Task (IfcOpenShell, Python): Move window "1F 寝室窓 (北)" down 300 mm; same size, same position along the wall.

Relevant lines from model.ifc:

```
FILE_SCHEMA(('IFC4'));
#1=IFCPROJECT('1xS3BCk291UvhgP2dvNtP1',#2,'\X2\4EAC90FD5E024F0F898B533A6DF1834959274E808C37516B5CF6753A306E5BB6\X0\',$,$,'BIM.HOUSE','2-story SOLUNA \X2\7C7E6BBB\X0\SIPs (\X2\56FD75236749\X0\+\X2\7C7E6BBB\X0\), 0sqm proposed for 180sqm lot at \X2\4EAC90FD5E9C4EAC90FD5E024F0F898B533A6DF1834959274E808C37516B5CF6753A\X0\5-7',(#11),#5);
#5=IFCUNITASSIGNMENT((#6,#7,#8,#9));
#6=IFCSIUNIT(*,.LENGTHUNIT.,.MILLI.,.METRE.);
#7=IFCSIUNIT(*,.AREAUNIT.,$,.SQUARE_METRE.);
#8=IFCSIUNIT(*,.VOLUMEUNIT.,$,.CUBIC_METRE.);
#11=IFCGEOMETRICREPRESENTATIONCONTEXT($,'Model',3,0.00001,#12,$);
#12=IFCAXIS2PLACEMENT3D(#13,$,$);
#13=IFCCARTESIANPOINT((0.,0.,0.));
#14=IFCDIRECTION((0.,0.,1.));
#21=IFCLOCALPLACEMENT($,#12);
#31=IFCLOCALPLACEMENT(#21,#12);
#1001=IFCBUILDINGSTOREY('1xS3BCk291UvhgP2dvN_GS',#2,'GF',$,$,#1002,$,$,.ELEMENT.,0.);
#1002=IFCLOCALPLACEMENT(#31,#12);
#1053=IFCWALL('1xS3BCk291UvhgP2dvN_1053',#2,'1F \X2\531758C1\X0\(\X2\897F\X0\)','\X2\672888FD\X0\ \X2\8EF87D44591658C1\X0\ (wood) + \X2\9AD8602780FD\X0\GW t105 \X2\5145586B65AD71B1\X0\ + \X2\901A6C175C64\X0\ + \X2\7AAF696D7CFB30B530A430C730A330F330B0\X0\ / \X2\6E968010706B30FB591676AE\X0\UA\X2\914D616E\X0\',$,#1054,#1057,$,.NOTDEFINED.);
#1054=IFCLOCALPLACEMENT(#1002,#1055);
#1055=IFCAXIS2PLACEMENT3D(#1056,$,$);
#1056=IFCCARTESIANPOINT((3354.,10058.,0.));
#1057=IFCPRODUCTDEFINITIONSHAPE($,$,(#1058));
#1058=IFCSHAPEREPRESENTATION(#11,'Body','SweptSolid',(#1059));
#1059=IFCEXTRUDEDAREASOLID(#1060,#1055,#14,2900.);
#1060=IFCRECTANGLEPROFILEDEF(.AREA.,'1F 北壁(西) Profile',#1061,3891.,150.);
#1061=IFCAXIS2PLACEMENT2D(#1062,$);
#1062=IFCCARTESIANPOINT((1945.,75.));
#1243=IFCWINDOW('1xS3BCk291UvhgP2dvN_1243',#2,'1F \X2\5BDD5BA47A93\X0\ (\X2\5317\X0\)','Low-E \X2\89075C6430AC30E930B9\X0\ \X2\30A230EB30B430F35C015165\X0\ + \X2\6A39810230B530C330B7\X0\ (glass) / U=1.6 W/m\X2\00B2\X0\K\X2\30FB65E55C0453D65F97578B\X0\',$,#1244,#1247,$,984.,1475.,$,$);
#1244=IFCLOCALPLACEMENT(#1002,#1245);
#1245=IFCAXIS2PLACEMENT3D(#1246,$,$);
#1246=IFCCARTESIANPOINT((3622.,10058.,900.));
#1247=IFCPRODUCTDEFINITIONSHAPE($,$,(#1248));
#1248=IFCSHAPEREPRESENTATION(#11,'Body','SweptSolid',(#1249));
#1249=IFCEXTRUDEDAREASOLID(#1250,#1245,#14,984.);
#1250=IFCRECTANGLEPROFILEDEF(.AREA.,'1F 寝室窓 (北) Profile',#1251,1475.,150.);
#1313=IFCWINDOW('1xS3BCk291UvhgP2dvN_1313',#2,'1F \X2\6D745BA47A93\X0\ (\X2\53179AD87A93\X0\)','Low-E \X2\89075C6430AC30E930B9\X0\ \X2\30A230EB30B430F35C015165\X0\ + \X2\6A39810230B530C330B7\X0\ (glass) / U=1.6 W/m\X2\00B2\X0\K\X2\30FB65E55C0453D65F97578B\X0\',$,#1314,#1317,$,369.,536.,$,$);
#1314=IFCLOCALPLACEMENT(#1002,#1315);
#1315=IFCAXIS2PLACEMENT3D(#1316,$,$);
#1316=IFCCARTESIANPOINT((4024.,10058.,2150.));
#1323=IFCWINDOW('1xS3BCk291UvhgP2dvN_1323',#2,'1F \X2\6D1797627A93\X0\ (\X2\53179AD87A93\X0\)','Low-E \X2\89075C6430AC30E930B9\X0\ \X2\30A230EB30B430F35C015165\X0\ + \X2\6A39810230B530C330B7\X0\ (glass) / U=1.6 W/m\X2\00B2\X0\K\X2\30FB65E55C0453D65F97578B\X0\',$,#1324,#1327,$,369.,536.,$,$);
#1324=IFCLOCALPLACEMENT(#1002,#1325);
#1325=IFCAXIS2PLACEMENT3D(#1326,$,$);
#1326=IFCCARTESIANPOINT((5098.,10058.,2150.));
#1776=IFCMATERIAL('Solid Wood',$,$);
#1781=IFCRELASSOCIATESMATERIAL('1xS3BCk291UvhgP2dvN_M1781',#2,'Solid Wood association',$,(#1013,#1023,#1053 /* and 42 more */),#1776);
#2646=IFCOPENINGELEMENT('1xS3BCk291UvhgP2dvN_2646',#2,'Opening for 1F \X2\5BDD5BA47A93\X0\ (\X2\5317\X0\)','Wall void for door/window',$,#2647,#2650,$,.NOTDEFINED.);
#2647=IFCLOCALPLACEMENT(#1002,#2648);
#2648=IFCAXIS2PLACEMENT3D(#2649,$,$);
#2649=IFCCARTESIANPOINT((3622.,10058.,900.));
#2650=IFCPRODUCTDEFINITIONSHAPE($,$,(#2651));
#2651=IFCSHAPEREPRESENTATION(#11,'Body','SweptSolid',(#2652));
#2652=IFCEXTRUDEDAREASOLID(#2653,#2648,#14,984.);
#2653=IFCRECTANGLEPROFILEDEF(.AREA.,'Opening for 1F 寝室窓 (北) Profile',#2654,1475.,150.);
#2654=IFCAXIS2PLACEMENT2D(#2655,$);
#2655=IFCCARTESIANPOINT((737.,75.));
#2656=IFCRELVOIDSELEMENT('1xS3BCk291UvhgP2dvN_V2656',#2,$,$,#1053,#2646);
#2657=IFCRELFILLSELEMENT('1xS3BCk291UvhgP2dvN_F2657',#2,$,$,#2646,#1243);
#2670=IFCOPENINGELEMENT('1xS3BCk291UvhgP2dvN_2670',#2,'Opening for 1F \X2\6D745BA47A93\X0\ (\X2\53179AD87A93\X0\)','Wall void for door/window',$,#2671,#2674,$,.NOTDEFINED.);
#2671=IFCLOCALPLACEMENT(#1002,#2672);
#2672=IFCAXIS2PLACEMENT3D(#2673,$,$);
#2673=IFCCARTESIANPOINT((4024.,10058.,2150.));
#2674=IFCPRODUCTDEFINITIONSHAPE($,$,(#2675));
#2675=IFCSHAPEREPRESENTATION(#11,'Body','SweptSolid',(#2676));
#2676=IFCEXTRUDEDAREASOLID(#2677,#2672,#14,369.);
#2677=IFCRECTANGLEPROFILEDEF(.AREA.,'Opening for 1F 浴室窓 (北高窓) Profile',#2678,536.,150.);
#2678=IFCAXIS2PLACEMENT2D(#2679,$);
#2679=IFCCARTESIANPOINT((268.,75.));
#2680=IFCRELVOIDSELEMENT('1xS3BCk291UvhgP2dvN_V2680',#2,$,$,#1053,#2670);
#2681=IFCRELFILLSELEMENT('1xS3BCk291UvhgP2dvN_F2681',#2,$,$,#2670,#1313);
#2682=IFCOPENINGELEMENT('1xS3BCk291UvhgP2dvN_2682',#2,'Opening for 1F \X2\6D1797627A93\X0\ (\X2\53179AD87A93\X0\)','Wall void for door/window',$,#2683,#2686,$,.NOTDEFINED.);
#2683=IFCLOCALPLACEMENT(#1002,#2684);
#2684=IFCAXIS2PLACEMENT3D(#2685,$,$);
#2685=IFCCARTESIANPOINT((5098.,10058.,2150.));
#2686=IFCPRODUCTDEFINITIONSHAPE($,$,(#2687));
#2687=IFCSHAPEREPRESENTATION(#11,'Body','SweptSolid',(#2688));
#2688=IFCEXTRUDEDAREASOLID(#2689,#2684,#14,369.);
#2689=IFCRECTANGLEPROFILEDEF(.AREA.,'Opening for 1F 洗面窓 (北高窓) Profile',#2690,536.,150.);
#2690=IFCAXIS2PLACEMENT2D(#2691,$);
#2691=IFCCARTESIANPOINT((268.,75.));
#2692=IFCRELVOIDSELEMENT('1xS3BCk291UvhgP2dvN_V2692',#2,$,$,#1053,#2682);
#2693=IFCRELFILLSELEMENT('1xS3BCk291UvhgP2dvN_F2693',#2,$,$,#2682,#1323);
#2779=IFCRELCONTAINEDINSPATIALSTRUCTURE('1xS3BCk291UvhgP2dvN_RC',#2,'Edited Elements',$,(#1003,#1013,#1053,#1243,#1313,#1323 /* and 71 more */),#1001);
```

```python
import numpy as np
import ifcopenshell
import ifcopenshell.api.geometry
import ifcopenshell.util.placement
import ifcopenshell.util.unit

model = ifcopenshell.open("model.ifc")
unit_scale = ifcopenshell.util.unit.calculate_unit_scale(model)

window = model.by_guid("1xS3BCk291UvhgP2dvN_1243")
opening = window.FillsVoids[0].RelatingOpeningElement
dz = -300.0

shift = np.array([0.0, 0.0, dz])
# The window is not placed relative to its opening, so move both.
for product in (opening, window):
    matrix = ifcopenshell.util.placement.get_local_placement(product.ObjectPlacement)
    matrix[:3, 3] += shift
    ifcopenshell.api.geometry.edit_object_placement(model, product=product, matrix=matrix, is_si=False)

print(f"moved by {dz * unit_scale:+.3f} m")

model.write("model_rev.ifc")
```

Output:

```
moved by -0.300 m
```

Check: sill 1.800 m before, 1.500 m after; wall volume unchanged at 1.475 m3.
